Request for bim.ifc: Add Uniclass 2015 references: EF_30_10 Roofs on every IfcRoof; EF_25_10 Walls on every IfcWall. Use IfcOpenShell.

First a look at what the model holds.

```python
import ifcopenshell

model = ifcopenshell.open("bim.ifc")
print(model.schema)
print("classifications:", [c.Name for c in model.by_type("IfcClassification")])
for ifc_class in ("IfcDoor", "IfcRoof", "IfcStair", "IfcWall", "IfcWindow"):
    print(ifc_class, len(model.by_type(ifc_class)))
```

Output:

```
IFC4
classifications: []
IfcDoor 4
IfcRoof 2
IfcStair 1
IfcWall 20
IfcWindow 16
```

```python
import ifcopenshell
import ifcopenshell.api.classification

model = ifcopenshell.open("bim.ifc")

system = ifcopenshell.api.classification.add_classification(model, classification="Uniclass 2015")

codes = {
    "IfcRoof": ("EF_30_10", "Roofs"),
    "IfcWall": ("EF_25_10", "Walls"),
}
for ifc_class, (code, name) in codes.items():
    products = model.by_type(ifc_class)
    ifcopenshell.api.classification.add_reference(
        model, products=products, classification=system, identification=code, name=name
    )
    print(code, len(products))

model.write("bim_v2.ifc")
```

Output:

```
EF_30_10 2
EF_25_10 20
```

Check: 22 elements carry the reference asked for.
